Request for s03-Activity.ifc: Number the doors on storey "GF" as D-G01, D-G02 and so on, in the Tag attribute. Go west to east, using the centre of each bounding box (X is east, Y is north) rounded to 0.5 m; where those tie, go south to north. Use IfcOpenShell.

First a look at what the model holds.

```python
import ifcopenshell
import ifcopenshell.util.element
import ifcopenshell.util.placement

model = ifcopenshell.open("s03-Activity.ifc")
print(model.schema)
storey = next(s for s in model.by_type("IfcBuildingStorey") if s.Name == "GF")
doors = [e for e in ifcopenshell.util.element.get_decomposition(storey) if e.is_a("IfcDoor")]
for e in sorted(doors, key=lambda e: e.id()):
    origin = ifcopenshell.util.placement.get_local_placement(e.ObjectPlacement)[:3, 3]
    print(e.id(), e.Tag, e.Name, origin.round(2) + 0.0, sep=" | ")
```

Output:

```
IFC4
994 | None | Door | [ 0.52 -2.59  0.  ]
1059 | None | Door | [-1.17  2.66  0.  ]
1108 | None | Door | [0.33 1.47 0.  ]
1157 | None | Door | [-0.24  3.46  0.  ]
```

```python
import ifcopenshell
import ifcopenshell.geom
import ifcopenshell.util.element
import ifcopenshell.util.shape

model = ifcopenshell.open("s03-Activity.ifc")
settings = ifcopenshell.geom.settings()
settings.set("use-world-coords", True)


def centre(element):
    shape = ifcopenshell.geom.create_shape(settings, element)
    return ifcopenshell.util.shape.get_bbox_centroid(shape.geometry)


storey = next(s for s in model.by_type("IfcBuildingStorey") if s.Name == "GF")
doors = [e for e in ifcopenshell.util.element.get_decomposition(storey) if e.is_a("IfcDoor")]

# Insertion points can sit at a corner or the storey origin, so sort by the geometry (in metres).
centres = {e: centre(e) for e in doors}
doors.sort(key=lambda e: (round(centres[e][0] / 0.5), centres[e][1]))

for i, e in enumerate(doors, start=1):
    number = f"D-G{i:02d}"
    e.Tag = number
    print(e.id(), number)

model.write("s03-Activity-out.ifc")
```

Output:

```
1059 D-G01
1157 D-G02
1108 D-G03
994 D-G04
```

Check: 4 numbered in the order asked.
